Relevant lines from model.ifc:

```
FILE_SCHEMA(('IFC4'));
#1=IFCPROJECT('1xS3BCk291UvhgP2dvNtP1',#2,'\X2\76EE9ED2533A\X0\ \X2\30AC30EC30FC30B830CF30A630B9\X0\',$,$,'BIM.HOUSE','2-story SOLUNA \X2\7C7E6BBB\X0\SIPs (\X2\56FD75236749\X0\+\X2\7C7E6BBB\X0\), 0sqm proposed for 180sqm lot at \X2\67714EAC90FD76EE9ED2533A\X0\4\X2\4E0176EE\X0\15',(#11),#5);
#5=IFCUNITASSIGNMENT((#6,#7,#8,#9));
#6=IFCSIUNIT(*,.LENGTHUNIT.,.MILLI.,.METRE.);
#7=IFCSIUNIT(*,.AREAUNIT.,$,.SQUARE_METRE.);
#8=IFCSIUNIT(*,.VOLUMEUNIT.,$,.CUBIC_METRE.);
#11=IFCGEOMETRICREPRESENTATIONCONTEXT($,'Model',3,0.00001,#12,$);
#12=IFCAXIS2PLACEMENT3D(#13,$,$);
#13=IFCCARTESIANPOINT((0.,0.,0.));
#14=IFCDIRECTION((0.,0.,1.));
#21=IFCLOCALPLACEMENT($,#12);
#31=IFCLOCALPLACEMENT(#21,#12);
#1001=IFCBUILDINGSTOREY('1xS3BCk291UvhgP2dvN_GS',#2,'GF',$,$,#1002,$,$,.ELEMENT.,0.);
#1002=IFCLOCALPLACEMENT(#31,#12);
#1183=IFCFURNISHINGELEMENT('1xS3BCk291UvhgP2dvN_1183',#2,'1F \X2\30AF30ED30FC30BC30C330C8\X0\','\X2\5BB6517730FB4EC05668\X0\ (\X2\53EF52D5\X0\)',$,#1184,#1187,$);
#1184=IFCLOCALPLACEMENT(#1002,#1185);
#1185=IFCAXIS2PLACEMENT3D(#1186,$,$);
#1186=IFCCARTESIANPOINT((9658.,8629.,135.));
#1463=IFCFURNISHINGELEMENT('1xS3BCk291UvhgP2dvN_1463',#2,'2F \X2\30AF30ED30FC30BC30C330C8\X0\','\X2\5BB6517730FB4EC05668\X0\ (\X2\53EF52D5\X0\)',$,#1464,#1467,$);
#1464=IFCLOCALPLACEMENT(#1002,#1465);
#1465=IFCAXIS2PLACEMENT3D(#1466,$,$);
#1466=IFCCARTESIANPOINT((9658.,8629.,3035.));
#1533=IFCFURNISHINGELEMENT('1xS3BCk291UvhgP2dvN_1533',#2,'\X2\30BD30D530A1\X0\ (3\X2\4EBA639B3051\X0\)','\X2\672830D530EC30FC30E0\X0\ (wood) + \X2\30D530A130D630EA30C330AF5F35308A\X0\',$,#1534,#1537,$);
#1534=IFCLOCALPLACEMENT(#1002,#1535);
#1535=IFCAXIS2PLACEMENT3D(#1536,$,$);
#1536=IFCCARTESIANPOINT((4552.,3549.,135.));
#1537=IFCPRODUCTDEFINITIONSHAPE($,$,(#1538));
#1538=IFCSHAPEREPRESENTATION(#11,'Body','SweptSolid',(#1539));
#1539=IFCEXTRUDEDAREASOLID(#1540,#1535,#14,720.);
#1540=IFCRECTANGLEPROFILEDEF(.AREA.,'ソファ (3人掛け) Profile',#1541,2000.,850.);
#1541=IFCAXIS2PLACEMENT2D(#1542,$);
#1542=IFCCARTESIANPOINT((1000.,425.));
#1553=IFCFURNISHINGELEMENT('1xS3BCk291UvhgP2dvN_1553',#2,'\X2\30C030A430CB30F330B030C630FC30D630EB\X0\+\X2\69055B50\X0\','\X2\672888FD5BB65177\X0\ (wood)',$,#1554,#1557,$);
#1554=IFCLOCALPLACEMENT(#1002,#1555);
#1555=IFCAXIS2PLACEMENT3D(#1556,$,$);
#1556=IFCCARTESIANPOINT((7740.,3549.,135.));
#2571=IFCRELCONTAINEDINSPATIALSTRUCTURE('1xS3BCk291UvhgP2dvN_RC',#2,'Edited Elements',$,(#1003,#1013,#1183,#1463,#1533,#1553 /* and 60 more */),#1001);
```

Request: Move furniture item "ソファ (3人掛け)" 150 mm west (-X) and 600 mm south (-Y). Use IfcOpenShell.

```python
import ifcopenshell
import ifcopenshell.api.geometry
import ifcopenshell.util.placement

model = ifcopenshell.open("model.ifc")

item = model.by_id(1533)
matrix = ifcopenshell.util.placement.get_local_placement(item.ObjectPlacement)
matrix[0, 3] -= 150.0
matrix[1, 3] -= 600.0
ifcopenshell.api.geometry.edit_object_placement(model, product=item, matrix=matrix, is_si=False)

print(ifcopenshell.util.placement.get_local_placement(item.ObjectPlacement).round(3) + 0.0)

model.write("model_edited.ifc")
```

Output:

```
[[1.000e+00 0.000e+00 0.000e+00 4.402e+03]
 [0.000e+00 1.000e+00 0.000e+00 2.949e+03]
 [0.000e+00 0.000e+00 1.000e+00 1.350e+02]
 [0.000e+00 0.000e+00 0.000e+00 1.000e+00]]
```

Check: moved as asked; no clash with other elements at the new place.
